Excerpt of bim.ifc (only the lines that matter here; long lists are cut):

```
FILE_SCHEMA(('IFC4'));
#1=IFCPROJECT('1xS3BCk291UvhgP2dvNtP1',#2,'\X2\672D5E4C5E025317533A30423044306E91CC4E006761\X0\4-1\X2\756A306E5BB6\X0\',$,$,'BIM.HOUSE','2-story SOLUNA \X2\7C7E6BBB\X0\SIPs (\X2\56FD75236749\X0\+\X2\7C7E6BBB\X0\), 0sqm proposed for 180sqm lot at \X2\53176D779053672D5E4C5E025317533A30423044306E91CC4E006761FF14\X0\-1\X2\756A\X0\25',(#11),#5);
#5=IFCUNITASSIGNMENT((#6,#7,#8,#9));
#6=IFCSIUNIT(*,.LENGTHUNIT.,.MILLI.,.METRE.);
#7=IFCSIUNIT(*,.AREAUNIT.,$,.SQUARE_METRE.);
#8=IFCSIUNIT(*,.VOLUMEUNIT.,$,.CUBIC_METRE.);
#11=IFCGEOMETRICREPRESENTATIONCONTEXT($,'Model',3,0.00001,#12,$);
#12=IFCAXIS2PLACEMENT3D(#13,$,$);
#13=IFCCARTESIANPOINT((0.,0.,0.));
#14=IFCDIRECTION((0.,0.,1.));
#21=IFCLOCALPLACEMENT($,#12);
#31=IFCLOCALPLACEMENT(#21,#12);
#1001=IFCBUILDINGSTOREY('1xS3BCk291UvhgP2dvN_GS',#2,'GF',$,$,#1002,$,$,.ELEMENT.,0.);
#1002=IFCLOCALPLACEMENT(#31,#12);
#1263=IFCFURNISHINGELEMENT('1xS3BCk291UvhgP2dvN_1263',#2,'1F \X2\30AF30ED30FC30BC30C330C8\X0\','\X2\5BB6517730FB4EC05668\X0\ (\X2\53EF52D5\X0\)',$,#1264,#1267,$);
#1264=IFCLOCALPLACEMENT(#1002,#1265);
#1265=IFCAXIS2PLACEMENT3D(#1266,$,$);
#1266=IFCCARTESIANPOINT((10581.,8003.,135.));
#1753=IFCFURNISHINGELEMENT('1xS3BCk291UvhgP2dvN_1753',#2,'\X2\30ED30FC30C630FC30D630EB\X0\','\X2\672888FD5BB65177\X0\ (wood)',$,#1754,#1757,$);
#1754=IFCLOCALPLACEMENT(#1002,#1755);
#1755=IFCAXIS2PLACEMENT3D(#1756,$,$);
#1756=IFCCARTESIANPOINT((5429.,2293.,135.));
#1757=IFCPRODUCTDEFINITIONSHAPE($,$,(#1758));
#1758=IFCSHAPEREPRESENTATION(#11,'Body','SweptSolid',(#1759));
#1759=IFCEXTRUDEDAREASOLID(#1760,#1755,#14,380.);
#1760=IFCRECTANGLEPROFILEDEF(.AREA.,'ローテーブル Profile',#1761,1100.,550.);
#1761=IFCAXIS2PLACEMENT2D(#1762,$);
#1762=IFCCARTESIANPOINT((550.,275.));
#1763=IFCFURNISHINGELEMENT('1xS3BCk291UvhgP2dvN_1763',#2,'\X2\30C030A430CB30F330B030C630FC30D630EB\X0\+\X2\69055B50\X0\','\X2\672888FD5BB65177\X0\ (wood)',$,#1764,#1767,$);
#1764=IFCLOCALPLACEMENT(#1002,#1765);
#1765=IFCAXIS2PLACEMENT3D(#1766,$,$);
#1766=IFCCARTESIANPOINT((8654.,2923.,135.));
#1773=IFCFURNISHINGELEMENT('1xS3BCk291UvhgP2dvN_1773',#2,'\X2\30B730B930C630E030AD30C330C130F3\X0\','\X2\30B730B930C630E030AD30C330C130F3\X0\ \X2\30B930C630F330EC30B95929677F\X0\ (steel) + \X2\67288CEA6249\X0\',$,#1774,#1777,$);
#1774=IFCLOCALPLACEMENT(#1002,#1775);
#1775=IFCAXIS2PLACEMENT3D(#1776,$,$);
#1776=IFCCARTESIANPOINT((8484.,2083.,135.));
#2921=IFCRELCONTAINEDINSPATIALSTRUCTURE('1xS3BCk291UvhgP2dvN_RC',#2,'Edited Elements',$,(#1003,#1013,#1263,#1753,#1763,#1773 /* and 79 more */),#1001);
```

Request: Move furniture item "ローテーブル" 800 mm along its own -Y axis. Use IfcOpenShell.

```python
import ifcopenshell
import ifcopenshell.api.geometry
import ifcopenshell.util.placement
import ifcopenshell.util.unit

model = ifcopenshell.open("bim.ifc")
unit_scale = ifcopenshell.util.unit.calculate_unit_scale(model)

item = model.by_guid("1xS3BCk291UvhgP2dvN_1753")
matrix = ifcopenshell.util.placement.get_local_placement(item.ObjectPlacement)
matrix[:3, 3] -= matrix[:3, 1] * 0.8 / unit_scale
ifcopenshell.api.geometry.edit_object_placement(model, product=item, matrix=matrix, is_si=False)

print(ifcopenshell.util.placement.get_local_placement(item.ObjectPlacement).round(3) + 0.0)

model.write("bim_updated.ifc")
```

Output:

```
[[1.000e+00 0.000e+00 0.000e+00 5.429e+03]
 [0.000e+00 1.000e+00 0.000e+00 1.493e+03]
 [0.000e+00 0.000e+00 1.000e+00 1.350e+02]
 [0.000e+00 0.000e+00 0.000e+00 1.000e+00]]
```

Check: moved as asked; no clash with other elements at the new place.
